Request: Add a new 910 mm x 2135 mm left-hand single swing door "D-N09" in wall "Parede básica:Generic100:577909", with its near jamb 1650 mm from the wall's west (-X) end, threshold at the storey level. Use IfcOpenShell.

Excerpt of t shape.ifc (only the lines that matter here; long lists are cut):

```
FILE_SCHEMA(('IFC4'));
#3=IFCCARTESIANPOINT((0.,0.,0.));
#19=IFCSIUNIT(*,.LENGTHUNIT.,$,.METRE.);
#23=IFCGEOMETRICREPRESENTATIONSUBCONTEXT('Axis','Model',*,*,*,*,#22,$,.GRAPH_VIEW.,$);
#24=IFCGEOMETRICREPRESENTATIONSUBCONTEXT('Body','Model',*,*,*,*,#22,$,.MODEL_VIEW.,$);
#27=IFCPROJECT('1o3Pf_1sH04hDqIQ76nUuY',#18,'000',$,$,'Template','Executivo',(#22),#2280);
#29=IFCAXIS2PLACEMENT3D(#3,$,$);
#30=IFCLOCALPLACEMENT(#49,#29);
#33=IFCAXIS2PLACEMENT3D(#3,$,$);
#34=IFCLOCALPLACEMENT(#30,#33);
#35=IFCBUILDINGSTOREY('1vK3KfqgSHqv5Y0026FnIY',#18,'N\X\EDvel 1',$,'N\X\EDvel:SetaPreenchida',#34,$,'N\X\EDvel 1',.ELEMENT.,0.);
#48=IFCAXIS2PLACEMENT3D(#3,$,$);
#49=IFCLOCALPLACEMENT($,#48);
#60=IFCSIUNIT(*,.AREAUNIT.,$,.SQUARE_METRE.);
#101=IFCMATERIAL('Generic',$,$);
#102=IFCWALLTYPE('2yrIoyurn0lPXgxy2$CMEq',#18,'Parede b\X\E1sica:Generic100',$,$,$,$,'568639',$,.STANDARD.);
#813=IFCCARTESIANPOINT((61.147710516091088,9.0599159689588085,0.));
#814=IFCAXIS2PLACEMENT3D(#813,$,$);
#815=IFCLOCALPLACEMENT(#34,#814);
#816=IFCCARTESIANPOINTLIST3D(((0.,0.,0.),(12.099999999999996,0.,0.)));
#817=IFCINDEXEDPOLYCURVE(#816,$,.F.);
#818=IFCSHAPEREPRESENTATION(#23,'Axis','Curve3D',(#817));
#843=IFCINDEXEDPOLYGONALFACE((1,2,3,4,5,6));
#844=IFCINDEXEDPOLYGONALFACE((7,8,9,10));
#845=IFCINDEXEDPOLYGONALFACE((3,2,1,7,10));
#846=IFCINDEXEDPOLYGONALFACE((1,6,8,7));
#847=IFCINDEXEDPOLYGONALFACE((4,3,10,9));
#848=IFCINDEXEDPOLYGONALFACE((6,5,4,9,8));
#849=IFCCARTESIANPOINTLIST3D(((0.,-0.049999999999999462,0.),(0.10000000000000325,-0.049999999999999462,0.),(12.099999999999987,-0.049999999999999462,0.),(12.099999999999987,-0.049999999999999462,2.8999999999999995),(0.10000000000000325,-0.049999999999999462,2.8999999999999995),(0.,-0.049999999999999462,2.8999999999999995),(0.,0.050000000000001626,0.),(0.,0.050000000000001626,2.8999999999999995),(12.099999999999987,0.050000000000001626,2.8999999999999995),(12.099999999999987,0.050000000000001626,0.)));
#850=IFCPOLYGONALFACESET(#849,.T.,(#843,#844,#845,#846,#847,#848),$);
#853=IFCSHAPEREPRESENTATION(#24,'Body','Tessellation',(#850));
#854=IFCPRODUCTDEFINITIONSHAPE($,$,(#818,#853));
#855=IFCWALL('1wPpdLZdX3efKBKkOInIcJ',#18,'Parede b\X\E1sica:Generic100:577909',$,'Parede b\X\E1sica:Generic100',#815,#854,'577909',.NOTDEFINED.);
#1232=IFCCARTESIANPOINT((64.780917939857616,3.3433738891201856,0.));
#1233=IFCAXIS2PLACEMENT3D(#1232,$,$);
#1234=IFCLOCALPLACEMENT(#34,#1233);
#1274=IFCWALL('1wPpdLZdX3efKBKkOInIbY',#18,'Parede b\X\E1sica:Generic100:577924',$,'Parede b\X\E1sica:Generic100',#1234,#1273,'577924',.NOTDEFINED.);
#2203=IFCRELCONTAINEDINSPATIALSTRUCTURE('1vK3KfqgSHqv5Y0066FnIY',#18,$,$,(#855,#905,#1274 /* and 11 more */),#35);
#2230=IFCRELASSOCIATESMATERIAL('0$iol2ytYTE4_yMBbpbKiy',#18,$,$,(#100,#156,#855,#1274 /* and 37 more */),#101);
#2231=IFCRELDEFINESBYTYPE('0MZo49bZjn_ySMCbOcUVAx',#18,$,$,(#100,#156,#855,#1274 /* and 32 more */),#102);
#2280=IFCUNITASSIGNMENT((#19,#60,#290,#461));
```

```python
import numpy as np
import ifcopenshell
import ifcopenshell.api.feature
import ifcopenshell.api.geometry
import ifcopenshell.api.root
import ifcopenshell.api.spatial
import ifcopenshell.geom
import ifcopenshell.util.element
import ifcopenshell.util.placement
import ifcopenshell.util.representation
import ifcopenshell.util.shape
import ifcopenshell.util.unit

model = ifcopenshell.open("t shape.ifc")
unit_scale = ifcopenshell.util.unit.calculate_unit_scale(model)
settings = ifcopenshell.geom.settings()


def volume(element):
    """Net volume in cubic metres, openings subtracted."""
    shape = ifcopenshell.geom.create_shape(settings, element)
    return ifcopenshell.util.shape.get_volume(shape.geometry)


wall = model.by_guid("1wPpdLZdX3efKBKkOInIcJ")
storey = ifcopenshell.util.element.get_container(wall, ifc_class="IfcBuildingStorey")
context = ifcopenshell.util.representation.get_context(model, "Model", "Body", "MODEL_VIEW")
before = volume(wall)

width, height, from_end, sill = 0.91, 2.135, 1.65, 0.0  # metres

# The wall runs along its own X axis, and the end named is its -X end.
wall_shape = ifcopenshell.geom.create_shape(settings, wall)
x, y, z = ifcopenshell.util.shape.get_vertices(wall_shape.geometry).T
start = x.min() + from_end
face, thickness = float(y.min()), float(y.max() - y.min())
wall_matrix = ifcopenshell.util.placement.get_local_placement(wall.ObjectPlacement)
level = ifcopenshell.util.placement.get_local_placement(storey.ObjectPlacement)[2, 3]


def in_wall(x, y):
    """Placement at x, y metres in the wall's axes, at sill height."""
    matrix = wall_matrix.copy()
    matrix[:, 3] = wall_matrix @ np.array([x / unit_scale, y / unit_scale, 0.0, 1.0])
    matrix[2, 3] = level + sill / unit_scale
    return matrix


# Opening: a box that overshoots both wall faces by 50 mm.
opening = ifcopenshell.api.root.create_entity(model, ifc_class="IfcOpeningElement", predefined_type="OPENING")
box = ifcopenshell.api.geometry.add_wall_representation(
    model, context=context, length=width, height=height, thickness=thickness + 0.1
)
ifcopenshell.api.geometry.assign_representation(model, product=opening, representation=box)
ifcopenshell.api.geometry.edit_object_placement(model, product=opening, matrix=in_wall(start, face - 0.05), is_si=False)
ifcopenshell.api.feature.add_feature(model, feature=opening, element=wall)

door = ifcopenshell.api.root.create_entity(model, ifc_class="IfcDoor", name="D-N09", predefined_type="DOOR")
door.OverallWidth, door.OverallHeight = width / unit_scale, height / unit_scale
door.OperationType = "SINGLE_SWING_LEFT"
body = ifcopenshell.api.geometry.add_door_representation(
    model,
    context=context,
    overall_width=door.OverallWidth,
    overall_height=door.OverallHeight,
    operation_type="SINGLE_SWING_LEFT",
    lining_properties={"LiningDepth": thickness / unit_scale, "ThresholdDepth": thickness / unit_scale},
)
ifcopenshell.api.geometry.assign_representation(model, product=door, representation=body)
ifcopenshell.api.spatial.assign_container(model, products=[door], relating_structure=storey)
ifcopenshell.api.feature.add_filling(model, opening=opening, element=door)

# The lining spans the wall, so the door starts at the wall face.
ifcopenshell.api.geometry.edit_object_placement(model, product=door, matrix=in_wall(start, face), is_si=False)

after = volume(wall)

print(f"wall volume {before:.3f} -> {after:.3f} m3")

model.write("t shape_v2.ifc")
```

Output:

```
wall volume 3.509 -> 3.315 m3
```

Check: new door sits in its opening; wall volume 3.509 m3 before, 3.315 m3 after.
